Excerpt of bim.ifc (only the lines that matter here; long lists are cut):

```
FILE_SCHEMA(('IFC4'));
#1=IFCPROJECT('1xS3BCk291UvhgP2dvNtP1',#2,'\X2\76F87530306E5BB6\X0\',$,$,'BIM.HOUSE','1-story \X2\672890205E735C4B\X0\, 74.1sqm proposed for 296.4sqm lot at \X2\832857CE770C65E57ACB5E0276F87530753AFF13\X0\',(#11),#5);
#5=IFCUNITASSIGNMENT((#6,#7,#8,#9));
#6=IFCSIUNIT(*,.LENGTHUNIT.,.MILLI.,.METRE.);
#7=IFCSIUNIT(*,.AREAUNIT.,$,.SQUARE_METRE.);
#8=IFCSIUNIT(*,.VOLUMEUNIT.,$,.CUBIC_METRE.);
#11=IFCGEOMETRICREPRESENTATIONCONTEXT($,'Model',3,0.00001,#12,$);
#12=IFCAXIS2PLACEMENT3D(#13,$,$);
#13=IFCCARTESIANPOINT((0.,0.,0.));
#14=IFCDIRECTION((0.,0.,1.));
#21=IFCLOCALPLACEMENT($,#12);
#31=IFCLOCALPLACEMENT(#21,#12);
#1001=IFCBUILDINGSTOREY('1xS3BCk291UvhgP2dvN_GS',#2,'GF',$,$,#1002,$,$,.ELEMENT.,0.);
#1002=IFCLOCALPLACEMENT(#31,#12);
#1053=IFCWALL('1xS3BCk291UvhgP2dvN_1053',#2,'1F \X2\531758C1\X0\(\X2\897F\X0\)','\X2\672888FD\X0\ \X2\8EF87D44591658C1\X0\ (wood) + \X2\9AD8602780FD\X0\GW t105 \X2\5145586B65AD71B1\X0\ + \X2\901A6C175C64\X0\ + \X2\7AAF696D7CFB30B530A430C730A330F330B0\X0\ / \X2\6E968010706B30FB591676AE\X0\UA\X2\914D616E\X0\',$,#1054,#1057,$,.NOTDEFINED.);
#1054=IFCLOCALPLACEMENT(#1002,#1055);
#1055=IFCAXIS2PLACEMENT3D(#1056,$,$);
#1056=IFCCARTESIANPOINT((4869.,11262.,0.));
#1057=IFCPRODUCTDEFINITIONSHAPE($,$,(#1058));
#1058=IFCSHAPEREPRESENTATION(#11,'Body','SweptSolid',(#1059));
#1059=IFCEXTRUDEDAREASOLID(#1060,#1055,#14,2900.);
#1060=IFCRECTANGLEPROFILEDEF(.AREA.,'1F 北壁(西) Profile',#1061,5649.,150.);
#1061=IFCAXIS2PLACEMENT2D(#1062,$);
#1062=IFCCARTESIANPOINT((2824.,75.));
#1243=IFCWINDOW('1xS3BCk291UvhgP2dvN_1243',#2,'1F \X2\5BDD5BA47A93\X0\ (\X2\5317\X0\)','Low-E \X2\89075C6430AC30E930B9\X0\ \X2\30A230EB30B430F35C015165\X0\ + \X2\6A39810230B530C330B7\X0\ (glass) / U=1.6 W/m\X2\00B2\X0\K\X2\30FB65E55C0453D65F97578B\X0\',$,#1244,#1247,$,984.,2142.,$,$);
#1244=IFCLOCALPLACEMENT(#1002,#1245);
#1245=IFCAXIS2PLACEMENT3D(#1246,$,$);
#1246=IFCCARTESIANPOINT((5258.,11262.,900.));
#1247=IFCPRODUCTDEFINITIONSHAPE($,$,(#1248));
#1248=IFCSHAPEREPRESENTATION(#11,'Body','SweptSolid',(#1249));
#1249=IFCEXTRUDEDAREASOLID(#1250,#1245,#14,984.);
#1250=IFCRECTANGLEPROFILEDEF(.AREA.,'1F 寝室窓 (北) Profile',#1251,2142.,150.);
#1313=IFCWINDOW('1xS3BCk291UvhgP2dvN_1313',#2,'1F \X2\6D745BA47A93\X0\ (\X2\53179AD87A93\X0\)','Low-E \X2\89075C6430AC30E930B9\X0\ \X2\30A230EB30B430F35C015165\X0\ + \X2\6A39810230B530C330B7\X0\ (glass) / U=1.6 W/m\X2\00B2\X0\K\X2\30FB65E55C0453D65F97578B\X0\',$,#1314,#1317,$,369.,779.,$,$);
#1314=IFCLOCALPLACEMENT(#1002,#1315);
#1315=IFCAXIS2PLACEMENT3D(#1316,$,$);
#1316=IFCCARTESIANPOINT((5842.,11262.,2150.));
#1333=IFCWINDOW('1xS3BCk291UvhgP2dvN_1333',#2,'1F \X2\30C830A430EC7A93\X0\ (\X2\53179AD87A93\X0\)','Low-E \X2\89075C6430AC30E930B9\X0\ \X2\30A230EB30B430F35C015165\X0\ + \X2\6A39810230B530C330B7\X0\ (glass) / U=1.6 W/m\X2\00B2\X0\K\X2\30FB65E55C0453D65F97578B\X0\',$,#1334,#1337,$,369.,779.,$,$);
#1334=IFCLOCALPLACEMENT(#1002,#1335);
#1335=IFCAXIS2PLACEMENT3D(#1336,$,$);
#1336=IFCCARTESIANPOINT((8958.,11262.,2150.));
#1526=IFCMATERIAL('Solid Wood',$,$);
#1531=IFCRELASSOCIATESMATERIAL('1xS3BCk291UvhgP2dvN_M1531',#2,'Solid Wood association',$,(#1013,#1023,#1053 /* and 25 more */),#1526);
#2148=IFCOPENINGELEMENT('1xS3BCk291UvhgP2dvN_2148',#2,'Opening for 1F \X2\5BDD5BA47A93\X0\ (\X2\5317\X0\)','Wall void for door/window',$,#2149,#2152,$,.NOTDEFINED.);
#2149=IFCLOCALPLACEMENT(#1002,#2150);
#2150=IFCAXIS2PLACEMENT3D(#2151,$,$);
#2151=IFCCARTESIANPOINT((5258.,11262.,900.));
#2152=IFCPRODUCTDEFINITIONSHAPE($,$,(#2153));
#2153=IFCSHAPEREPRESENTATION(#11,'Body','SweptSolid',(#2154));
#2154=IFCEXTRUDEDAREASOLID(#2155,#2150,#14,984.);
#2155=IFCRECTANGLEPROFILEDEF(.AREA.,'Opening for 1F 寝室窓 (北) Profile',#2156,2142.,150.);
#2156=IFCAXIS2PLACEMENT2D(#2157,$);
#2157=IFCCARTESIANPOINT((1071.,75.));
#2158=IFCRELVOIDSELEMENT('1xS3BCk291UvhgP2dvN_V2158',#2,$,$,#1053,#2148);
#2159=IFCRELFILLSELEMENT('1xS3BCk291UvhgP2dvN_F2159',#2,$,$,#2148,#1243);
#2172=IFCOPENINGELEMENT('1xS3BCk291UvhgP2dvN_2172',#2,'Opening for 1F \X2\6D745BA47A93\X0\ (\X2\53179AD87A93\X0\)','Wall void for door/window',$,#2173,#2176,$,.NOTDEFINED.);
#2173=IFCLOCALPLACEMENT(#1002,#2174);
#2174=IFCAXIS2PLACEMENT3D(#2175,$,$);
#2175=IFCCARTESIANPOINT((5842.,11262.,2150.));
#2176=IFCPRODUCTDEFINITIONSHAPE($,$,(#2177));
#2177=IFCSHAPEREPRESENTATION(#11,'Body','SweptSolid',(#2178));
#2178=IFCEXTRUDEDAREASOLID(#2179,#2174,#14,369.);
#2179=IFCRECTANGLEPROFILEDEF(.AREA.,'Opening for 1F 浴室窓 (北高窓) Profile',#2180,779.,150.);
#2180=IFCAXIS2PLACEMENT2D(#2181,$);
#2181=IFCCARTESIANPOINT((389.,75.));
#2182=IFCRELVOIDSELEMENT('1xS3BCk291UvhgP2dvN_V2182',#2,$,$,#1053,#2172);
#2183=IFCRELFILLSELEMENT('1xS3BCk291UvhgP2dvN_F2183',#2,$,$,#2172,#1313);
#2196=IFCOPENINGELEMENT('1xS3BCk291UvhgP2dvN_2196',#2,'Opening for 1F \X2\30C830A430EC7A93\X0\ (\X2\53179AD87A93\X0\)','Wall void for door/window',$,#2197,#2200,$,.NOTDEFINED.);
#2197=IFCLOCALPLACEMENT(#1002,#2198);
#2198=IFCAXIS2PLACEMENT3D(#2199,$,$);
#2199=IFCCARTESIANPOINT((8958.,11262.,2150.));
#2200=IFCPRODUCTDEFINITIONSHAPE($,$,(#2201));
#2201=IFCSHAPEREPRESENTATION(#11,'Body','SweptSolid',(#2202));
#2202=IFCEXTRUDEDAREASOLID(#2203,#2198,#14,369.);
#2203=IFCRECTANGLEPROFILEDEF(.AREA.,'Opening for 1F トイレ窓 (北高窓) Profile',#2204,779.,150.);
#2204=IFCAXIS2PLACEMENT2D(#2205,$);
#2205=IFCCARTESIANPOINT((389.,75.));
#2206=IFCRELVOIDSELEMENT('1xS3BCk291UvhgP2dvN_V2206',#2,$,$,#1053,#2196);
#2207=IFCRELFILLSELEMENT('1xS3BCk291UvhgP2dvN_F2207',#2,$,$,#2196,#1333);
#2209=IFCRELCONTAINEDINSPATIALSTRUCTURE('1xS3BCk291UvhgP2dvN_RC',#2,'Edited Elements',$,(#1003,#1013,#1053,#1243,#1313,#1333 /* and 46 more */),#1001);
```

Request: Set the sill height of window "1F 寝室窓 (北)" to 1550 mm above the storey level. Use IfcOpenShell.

```python
import numpy as np
import ifcopenshell
import ifcopenshell.api.geometry
import ifcopenshell.geom
import ifcopenshell.util.element
import ifcopenshell.util.placement
import ifcopenshell.util.shape
import ifcopenshell.util.unit

model = ifcopenshell.open("bim.ifc")
unit_scale = ifcopenshell.util.unit.calculate_unit_scale(model)

window = model.by_id(1243)
opening = window.FillsVoids[0].RelatingOpeningElement
storey = ifcopenshell.util.element.get_container(window, ifc_class="IfcBuildingStorey")
level = ifcopenshell.util.placement.get_local_placement(storey.ObjectPlacement)[2, 3]

# The opening's origin need not be at the sill, so measure its lowest point.
shape = ifcopenshell.geom.create_shape(ifcopenshell.geom.settings(), opening)
bottom = ifcopenshell.util.shape.get_shape_bottom_elevation(shape, shape.geometry) / unit_scale
dz = level + 1.55 / unit_scale - bottom

shift = np.array([0.0, 0.0, dz])
# The window is not placed relative to its opening, so move both.
for product in (opening, window):
    matrix = ifcopenshell.util.placement.get_local_placement(product.ObjectPlacement)
    matrix[:3, 3] += shift
    ifcopenshell.api.geometry.edit_object_placement(model, product=product, matrix=matrix, is_si=False)

print(f"moved by {dz * unit_scale:+.3f} m")

model.write("bim_edited.ifc")
```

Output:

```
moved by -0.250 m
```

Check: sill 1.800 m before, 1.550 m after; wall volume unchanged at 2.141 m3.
